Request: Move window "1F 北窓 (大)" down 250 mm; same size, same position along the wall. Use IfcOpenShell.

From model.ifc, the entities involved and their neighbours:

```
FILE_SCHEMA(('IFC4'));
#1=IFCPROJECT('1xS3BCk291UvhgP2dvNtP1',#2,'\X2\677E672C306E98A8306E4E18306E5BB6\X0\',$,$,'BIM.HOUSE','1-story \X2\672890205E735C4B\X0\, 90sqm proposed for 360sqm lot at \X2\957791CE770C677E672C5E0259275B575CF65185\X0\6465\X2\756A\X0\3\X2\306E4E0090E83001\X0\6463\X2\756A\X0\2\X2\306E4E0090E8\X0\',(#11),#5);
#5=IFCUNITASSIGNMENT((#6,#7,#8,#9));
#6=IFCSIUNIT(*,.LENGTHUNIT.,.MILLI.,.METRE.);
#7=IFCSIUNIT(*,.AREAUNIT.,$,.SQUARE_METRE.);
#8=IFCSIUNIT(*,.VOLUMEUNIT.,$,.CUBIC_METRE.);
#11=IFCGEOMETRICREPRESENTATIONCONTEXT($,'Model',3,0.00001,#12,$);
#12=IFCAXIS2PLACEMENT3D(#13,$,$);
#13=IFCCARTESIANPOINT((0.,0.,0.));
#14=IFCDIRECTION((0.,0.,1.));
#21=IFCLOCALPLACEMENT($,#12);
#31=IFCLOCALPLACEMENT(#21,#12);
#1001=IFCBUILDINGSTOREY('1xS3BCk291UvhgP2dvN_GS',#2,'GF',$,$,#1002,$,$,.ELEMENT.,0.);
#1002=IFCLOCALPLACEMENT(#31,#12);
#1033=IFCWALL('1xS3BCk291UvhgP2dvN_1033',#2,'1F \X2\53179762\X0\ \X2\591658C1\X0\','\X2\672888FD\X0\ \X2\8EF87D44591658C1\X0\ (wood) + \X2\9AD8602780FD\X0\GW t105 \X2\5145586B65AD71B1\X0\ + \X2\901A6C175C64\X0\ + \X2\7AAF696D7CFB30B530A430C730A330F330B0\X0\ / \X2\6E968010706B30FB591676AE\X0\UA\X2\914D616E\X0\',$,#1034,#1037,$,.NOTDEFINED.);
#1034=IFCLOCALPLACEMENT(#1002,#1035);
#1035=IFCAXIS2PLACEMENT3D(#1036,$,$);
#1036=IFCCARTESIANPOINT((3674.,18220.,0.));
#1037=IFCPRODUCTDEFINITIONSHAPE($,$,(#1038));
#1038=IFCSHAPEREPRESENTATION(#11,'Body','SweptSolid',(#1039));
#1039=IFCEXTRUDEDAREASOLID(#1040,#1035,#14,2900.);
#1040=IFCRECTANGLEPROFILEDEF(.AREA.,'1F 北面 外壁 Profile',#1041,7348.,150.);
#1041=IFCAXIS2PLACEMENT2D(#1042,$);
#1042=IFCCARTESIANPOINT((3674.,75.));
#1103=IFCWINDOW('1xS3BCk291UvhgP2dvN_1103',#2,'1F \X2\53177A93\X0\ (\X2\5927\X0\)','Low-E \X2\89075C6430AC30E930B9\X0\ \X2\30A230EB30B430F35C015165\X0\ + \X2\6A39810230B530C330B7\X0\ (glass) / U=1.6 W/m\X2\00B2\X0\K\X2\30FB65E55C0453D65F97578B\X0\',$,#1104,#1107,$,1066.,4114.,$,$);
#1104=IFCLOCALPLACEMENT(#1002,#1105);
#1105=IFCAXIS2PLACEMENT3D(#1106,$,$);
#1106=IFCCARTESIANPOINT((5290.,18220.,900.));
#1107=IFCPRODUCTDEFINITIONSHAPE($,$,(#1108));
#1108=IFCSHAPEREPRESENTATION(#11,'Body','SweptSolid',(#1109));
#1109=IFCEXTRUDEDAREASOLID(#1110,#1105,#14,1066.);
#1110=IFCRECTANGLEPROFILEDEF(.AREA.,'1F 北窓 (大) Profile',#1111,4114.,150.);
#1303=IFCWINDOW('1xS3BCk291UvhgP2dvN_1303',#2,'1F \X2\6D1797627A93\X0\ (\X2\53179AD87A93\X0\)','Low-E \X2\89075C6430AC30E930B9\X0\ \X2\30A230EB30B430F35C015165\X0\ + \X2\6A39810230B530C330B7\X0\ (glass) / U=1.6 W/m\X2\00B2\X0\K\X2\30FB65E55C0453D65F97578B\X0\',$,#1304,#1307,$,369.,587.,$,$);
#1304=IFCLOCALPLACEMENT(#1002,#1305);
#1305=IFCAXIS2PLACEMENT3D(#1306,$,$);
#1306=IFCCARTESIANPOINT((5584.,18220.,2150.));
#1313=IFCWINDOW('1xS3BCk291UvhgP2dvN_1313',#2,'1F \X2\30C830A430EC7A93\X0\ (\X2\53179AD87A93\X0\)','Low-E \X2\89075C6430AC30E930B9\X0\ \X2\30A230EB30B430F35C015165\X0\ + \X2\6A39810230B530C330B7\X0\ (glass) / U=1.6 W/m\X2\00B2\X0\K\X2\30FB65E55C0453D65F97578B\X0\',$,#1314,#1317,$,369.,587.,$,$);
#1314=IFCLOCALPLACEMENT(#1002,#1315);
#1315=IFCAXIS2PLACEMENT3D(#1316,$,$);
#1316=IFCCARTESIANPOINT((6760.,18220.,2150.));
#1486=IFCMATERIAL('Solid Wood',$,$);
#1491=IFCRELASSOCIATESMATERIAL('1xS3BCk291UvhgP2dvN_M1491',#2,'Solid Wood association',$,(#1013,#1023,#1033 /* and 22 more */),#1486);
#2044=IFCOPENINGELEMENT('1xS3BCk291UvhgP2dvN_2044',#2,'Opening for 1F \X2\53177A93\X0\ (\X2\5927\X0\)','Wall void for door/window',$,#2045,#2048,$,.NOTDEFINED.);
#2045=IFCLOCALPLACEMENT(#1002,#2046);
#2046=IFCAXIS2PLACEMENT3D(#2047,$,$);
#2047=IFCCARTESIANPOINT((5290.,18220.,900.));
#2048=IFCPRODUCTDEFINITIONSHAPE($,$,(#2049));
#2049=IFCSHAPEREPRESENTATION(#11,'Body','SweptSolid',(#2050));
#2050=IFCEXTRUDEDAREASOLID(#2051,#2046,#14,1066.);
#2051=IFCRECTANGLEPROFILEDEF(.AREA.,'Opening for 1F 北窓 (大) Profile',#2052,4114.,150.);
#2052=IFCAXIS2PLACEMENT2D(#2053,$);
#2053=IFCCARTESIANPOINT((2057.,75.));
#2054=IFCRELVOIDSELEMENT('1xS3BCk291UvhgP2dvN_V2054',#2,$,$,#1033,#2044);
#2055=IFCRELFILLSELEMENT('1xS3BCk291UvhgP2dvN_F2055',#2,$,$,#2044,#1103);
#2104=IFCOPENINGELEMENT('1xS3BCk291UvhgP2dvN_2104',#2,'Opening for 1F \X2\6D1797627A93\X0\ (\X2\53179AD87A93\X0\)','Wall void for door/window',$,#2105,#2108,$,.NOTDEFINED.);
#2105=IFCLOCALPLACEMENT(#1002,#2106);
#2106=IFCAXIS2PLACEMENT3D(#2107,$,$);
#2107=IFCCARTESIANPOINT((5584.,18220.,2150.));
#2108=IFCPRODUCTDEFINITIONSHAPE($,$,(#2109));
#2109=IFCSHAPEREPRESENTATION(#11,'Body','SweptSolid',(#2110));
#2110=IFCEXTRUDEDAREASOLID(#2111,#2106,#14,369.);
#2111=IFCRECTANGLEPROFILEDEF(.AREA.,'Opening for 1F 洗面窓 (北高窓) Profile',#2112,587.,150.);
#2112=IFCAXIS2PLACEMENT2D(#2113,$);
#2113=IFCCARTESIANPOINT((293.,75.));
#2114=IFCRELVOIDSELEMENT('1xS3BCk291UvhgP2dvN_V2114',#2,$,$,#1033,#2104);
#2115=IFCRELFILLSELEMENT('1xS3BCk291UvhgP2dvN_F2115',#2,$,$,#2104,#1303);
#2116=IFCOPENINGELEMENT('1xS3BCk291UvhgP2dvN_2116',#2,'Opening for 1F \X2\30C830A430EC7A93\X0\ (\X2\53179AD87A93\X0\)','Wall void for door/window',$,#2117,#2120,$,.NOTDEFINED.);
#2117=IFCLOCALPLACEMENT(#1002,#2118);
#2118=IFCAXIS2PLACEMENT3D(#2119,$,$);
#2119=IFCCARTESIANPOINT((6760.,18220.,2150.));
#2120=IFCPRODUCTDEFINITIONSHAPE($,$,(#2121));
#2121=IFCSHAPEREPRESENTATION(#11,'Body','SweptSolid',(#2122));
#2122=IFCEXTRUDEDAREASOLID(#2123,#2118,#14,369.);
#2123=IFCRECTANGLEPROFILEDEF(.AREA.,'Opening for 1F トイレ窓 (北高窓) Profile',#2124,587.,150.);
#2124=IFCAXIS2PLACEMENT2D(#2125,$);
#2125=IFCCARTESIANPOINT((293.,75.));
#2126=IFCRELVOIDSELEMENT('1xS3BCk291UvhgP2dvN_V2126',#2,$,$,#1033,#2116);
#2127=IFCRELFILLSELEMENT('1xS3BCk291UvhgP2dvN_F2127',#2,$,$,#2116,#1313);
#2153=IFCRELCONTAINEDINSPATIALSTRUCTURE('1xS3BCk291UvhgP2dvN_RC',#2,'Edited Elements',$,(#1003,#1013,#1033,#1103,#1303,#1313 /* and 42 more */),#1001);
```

```python
import numpy as np
import ifcopenshell
import ifcopenshell.api.geometry
import ifcopenshell.util.placement
import ifcopenshell.util.unit

model = ifcopenshell.open("model.ifc")
unit_scale = ifcopenshell.util.unit.calculate_unit_scale(model)

window = model.by_guid("1xS3BCk291UvhgP2dvN_1103")
opening = window.FillsVoids[0].RelatingOpeningElement
dz = -0.25 / unit_scale

shift = np.array([0.0, 0.0, dz])
# The window is not placed relative to its opening, so move both.
for product in (opening, window):
    matrix = ifcopenshell.util.placement.get_local_placement(product.ObjectPlacement)
    matrix[:3, 3] += shift
    ifcopenshell.api.geometry.edit_object_placement(model, product=product, matrix=matrix, is_si=False)

print(f"moved by {dz * unit_scale:+.3f} m")

model.write("model_updated.ifc")
```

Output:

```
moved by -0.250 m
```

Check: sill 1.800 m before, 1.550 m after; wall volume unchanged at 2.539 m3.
